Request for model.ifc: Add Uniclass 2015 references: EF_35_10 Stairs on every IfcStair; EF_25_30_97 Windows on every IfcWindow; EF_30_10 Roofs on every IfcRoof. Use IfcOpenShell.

First a look at what the model holds.

```python
import ifcopenshell

model = ifcopenshell.open("model.ifc")
print(model.schema)
print("classifications:", [c.Name for c in model.by_type("IfcClassification")])
for ifc_class in ("IfcDoor", "IfcRoof", "IfcStair", "IfcWall", "IfcWindow"):
    print(ifc_class, len(model.by_type(ifc_class)))
```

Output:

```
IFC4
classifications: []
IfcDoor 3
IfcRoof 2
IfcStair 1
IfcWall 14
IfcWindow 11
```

```python
import ifcopenshell
import ifcopenshell.api.classification

model = ifcopenshell.open("model.ifc")

system = ifcopenshell.api.classification.add_classification(model, classification="Uniclass 2015")

codes = {
    "IfcStair": ("EF_35_10", "Stairs"),
    "IfcWindow": ("EF_25_30_97", "Windows"),
    "IfcRoof": ("EF_30_10", "Roofs"),
}
for ifc_class, (code, name) in codes.items():
    products = model.by_type(ifc_class)
    ifcopenshell.api.classification.add_reference(
        model, products=products, classification=system, identification=code, name=name
    )
    print(code, len(products))

model.write("model_updated.ifc")
```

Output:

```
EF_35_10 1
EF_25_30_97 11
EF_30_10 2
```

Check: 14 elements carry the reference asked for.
